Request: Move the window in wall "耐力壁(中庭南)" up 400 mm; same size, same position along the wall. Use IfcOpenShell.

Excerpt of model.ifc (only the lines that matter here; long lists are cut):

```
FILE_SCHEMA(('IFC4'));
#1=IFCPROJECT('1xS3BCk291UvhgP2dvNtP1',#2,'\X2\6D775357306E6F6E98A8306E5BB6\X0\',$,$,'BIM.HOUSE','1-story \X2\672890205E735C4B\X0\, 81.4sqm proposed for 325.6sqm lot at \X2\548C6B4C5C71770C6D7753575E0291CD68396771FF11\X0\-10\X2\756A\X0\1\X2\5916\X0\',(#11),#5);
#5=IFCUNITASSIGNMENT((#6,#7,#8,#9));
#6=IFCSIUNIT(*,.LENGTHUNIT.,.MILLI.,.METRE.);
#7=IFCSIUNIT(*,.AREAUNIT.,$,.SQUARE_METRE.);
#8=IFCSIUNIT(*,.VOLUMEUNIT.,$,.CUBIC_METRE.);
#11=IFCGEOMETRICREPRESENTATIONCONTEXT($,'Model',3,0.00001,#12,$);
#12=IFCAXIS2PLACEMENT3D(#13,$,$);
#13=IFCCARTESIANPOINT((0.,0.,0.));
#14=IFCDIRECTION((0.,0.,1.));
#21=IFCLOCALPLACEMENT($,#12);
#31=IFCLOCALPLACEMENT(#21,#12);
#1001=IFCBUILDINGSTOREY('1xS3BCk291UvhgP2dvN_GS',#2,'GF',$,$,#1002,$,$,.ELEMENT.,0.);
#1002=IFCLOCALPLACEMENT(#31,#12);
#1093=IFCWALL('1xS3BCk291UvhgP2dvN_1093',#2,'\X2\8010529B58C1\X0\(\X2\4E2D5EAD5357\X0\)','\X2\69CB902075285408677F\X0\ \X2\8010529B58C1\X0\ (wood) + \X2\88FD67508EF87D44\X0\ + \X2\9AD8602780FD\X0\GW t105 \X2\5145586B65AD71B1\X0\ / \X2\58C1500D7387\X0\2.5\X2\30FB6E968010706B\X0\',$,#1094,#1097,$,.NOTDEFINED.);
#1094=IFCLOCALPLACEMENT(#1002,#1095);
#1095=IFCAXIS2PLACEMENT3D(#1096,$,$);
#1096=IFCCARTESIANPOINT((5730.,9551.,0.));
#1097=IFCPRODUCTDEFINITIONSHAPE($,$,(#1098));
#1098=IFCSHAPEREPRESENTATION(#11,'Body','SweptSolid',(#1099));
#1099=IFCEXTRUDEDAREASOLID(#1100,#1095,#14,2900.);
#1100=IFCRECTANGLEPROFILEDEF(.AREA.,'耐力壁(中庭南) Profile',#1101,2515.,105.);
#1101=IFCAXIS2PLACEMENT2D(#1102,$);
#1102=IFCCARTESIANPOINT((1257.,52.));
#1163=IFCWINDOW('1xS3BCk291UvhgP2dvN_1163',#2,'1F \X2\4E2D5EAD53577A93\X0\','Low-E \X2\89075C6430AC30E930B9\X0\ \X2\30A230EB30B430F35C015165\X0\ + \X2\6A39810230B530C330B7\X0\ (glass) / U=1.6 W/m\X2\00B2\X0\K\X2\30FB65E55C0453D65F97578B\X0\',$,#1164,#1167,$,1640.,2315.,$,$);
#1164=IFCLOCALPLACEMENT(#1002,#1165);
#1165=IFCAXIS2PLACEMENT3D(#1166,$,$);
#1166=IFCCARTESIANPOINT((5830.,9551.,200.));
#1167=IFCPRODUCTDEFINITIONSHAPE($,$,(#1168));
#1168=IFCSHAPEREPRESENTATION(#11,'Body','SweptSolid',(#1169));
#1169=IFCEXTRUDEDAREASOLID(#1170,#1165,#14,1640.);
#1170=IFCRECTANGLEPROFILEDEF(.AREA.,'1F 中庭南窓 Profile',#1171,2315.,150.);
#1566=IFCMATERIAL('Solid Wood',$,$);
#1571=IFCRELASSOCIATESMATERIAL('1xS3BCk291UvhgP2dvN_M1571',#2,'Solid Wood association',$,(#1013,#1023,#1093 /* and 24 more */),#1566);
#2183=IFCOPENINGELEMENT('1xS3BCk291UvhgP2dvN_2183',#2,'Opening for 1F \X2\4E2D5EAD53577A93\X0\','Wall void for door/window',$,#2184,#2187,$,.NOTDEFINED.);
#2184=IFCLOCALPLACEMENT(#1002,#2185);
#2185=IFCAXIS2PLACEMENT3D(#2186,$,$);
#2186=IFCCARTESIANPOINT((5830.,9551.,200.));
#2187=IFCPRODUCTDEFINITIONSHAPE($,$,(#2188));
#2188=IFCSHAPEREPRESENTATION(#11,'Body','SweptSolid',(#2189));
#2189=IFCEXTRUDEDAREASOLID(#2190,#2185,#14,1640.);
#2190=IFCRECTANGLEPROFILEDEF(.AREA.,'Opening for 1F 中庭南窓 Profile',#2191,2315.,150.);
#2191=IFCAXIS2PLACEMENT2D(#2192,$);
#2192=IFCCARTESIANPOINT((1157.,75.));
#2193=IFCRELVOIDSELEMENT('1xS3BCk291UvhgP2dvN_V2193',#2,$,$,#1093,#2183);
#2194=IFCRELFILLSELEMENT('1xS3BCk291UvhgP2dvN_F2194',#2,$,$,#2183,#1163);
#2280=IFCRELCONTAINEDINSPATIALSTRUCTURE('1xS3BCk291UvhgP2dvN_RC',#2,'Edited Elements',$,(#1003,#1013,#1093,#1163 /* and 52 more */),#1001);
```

```python
import numpy as np
import ifcopenshell
import ifcopenshell.api.geometry
import ifcopenshell.util.placement
import ifcopenshell.util.unit

model = ifcopenshell.open("model.ifc")
unit_scale = ifcopenshell.util.unit.calculate_unit_scale(model)

window = model.by_id(1163)
opening = window.FillsVoids[0].RelatingOpeningElement
dz = 400.0

shift = np.array([0.0, 0.0, dz])
# The window is not placed relative to its opening, so move both.
for product in (opening, window):
    matrix = ifcopenshell.util.placement.get_local_placement(product.ObjectPlacement)
    matrix[:3, 3] += shift
    ifcopenshell.api.geometry.edit_object_placement(model, product=product, matrix=matrix, is_si=False)

print(f"moved by {dz * unit_scale:+.3f} m")

model.write("model-out.ifc")
```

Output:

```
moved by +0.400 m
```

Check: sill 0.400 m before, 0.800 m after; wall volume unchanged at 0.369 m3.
